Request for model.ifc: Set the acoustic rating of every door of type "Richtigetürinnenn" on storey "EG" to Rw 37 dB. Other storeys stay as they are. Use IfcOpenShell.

First a look at what the model holds.

```python
import ifcopenshell
import ifcopenshell.util.element

model = ifcopenshell.open("model.ifc")
print(model.schema)
storey = next(s for s in model.by_type("IfcBuildingStorey") if s.Name == "EG")
doors = [e for e in ifcopenshell.util.element.get_decomposition(storey) if e.is_a("IfcDoor")]
seen = {}
for e in doors:
    element_type = ifcopenshell.util.element.get_type(e)
    key = (element_type.Name if element_type != e and element_type else None, ifcopenshell.util.element.get_pset(e, "Pset_DoorCommon", "AcousticRating"))
    seen[key] = seen.get(key, 0) + 1
for (name, value), count in sorted(seen.items(), key=str):
    print(count, "x", name, "|", value)
```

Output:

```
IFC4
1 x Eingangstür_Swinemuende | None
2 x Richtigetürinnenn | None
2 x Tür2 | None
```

```python
import ifcopenshell
import ifcopenshell.api.pset
import ifcopenshell.util.element

model = ifcopenshell.open("model.ifc")

storey = next(s for s in model.by_type("IfcBuildingStorey") if s.Name == "EG")
doors = [e for e in ifcopenshell.util.element.get_decomposition(storey) if e.is_a("IfcDoor")]

count = 0
for e in doors:
    element_type = ifcopenshell.util.element.get_type(e)
    if element_type in (None, e) or element_type.Name != "Richtigetürinnenn":
        continue
    # add_pset returns the element's existing set when there is one.
    pset = ifcopenshell.api.pset.add_pset(model, product=e, name="Pset_DoorCommon")
    ifcopenshell.api.pset.edit_pset(model, pset=pset, properties={"AcousticRating": "Rw 37 dB"})
    count += 1

print(count, "doors updated")

model.write("model_edited.ifc")
```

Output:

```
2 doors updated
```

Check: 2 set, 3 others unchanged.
